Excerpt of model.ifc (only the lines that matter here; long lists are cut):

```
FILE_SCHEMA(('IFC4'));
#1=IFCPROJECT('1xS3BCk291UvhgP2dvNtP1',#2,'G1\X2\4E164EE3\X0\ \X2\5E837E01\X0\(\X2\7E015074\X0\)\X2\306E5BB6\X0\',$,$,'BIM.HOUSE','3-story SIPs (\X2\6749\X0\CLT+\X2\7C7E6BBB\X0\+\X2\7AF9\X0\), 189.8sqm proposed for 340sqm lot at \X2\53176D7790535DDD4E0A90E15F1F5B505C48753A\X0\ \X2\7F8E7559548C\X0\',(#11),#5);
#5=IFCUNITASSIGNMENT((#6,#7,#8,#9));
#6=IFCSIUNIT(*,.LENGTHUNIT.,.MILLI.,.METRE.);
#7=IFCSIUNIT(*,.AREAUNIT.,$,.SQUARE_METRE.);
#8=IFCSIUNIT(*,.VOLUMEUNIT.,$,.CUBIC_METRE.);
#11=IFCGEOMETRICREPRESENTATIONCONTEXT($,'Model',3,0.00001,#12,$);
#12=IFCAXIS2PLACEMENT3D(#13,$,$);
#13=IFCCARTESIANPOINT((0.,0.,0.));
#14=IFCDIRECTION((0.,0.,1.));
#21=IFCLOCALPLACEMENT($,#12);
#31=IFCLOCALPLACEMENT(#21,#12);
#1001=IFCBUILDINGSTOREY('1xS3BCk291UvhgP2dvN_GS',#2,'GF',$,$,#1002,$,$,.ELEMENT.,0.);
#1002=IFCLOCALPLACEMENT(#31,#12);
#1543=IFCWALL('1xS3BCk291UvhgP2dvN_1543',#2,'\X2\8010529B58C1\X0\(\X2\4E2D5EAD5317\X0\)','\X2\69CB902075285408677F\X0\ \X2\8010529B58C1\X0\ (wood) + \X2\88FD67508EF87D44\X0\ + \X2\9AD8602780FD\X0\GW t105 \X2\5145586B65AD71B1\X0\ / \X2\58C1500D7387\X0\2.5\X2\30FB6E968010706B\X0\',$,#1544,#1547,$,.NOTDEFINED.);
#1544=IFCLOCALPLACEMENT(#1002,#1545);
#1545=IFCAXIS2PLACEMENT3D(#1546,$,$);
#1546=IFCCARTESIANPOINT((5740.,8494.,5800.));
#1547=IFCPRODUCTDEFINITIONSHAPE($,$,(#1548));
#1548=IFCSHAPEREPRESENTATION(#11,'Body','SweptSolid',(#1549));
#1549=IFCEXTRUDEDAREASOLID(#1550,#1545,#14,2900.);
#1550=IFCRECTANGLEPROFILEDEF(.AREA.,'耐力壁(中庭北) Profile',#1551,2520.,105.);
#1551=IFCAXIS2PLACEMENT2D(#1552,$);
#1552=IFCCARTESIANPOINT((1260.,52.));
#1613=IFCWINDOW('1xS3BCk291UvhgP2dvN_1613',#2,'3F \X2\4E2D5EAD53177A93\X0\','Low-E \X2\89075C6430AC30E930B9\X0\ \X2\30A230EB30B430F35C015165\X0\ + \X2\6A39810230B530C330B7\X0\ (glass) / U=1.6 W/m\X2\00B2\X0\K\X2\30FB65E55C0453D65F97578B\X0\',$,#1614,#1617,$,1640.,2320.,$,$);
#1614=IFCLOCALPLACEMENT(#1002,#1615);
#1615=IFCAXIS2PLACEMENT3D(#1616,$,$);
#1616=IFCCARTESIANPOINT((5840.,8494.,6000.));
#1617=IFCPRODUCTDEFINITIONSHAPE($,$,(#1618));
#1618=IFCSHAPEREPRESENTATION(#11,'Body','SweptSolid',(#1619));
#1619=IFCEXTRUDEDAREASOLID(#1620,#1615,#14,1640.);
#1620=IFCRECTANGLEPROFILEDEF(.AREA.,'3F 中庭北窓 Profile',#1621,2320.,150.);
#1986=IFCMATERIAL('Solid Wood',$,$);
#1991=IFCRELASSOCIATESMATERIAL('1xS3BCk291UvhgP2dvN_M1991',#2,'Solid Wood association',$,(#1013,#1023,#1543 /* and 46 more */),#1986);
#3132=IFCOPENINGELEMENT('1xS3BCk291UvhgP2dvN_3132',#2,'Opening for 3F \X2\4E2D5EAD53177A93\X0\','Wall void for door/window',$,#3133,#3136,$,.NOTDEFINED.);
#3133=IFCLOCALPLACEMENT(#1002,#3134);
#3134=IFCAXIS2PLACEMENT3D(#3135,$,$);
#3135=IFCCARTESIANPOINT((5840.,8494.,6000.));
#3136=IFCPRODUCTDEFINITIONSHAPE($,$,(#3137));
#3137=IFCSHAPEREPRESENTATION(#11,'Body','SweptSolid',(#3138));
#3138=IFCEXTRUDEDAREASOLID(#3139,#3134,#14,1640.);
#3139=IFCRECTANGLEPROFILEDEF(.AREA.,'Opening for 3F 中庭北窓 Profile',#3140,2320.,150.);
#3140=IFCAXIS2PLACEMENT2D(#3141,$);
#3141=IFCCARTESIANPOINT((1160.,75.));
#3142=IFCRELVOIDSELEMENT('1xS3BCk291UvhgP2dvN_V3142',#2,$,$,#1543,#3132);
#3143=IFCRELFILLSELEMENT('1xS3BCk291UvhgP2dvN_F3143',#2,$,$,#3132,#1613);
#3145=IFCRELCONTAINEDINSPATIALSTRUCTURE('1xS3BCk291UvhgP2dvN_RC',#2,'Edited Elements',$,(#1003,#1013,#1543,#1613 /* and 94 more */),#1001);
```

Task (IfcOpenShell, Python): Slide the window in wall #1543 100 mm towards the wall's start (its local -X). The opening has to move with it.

```python
import ifcopenshell
import ifcopenshell.api.geometry
import ifcopenshell.util.placement
import ifcopenshell.util.unit

model = ifcopenshell.open("model.ifc")
unit_scale = ifcopenshell.util.unit.calculate_unit_scale(model)

window = model.by_guid("1xS3BCk291UvhgP2dvN_1613")
opening = window.FillsVoids[0].RelatingOpeningElement
wall = opening.VoidsElements[0].RelatingBuildingElement

wall_matrix = ifcopenshell.util.placement.get_local_placement(wall.ObjectPlacement)
shift = wall_matrix[:3, 0] * -0.1 / unit_scale
before = ifcopenshell.util.placement.get_local_placement(window.ObjectPlacement)[:3, 3].copy()

# The window is not placed relative to its opening, so move both.
for product in (opening, window):
    matrix = ifcopenshell.util.placement.get_local_placement(product.ObjectPlacement)
    matrix[:3, 3] += shift
    ifcopenshell.api.geometry.edit_object_placement(model, product=product, matrix=matrix, is_si=False)

after = ifcopenshell.util.placement.get_local_placement(window.ObjectPlacement)[:3, 3]
print("window moved by", (after - before).round(3) + 0.0)

model.write("model_updated.ifc")
```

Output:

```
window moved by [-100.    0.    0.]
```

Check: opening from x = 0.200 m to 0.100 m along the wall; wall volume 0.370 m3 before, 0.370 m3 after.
